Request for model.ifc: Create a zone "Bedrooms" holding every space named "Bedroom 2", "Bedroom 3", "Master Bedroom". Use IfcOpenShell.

First a look at what the model holds.

```python
import ifcopenshell

model = ifcopenshell.open("model.ifc")
print(model.schema)
seen = {}
for space in model.by_type("IfcSpace"):
    seen[space.LongName] = seen.get(space.LongName, 0) + 1
for name, count in sorted(seen.items(), key=str):
    print(count, "x", name)
print("zones:", [z.Name for z in model.by_type("IfcZone")][:20])
```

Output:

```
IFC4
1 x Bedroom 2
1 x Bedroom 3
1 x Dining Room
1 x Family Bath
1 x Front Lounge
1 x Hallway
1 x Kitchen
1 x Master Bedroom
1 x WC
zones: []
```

```python
import ifcopenshell
import ifcopenshell.api.group
import ifcopenshell.api.root

model = ifcopenshell.open("model.ifc")

names = {"Bedroom 2", "Bedroom 3", "Master Bedroom"}
spaces = [s for s in model.by_type("IfcSpace") if s.LongName in names]

zone = ifcopenshell.api.root.create_entity(model, ifc_class="IfcZone", name="Bedrooms")
ifcopenshell.api.group.assign_group(model, products=spaces, group=zone)
print(len(spaces), "spaces in", zone.Name)

model.write("model_edited.ifc")
```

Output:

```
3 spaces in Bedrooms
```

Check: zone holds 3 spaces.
